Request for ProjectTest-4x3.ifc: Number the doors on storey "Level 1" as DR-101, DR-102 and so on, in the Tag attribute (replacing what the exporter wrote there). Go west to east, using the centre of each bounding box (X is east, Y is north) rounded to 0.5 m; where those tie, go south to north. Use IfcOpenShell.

First a look at what the model holds.

```python
import ifcopenshell
import ifcopenshell.util.element
import ifcopenshell.util.placement

model = ifcopenshell.open("ProjectTest-4x3.ifc")
print(model.schema)
storey = next(s for s in model.by_type("IfcBuildingStorey") if s.Name == "Level 1")
doors = [e for e in ifcopenshell.util.element.get_decomposition(storey) if e.is_a("IfcDoor")]
for e in sorted(doors, key=lambda e: e.id()):
    origin = ifcopenshell.util.placement.get_local_placement(e.ObjectPlacement)[:3, 3]
    print(e.id(), e.Tag, e.Name, origin.round(2) + 0.0, sep=" | ")
```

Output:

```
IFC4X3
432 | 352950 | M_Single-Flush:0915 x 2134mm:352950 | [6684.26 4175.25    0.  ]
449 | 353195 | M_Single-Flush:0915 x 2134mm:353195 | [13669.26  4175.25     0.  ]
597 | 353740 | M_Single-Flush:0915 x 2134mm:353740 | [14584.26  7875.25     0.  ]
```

```python
import ifcopenshell
import ifcopenshell.geom
import ifcopenshell.util.element
import ifcopenshell.util.shape

model = ifcopenshell.open("ProjectTest-4x3.ifc")
settings = ifcopenshell.geom.settings()
settings.set("use-world-coords", True)


def centre(element):
    shape = ifcopenshell.geom.create_shape(settings, element)
    return ifcopenshell.util.shape.get_bbox_centroid(shape.geometry)


storey = next(s for s in model.by_type("IfcBuildingStorey") if s.Name == "Level 1")
doors = [e for e in ifcopenshell.util.element.get_decomposition(storey) if e.is_a("IfcDoor")]

# Insertion points can sit at a corner or the storey origin, so sort by the geometry (in metres).
centres = {e: centre(e) for e in doors}
doors.sort(key=lambda e: (round(centres[e][0] / 0.5), centres[e][1]))

for i, e in enumerate(doors, start=1):
    number = f"DR-1{i:02d}"
    e.Tag = number
    print(e.id(), number)

model.write("ProjectTest-4x3_edited.ifc")
```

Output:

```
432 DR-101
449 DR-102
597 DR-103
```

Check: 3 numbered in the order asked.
